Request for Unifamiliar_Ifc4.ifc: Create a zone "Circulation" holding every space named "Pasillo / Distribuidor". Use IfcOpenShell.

First a look at what the model holds.

```python
import ifcopenshell

model = ifcopenshell.open("Unifamiliar_Ifc4.ifc")
print(model.schema)
seen = {}
for space in model.by_type("IfcSpace"):
    seen[space.LongName] = seen.get(space.LongName, 0) + 1
for name, count in sorted(seen.items(), key=str):
    print(count, "x", name)
print("zones:", [z.Name for z in model.by_type("IfcZone")][:20])
```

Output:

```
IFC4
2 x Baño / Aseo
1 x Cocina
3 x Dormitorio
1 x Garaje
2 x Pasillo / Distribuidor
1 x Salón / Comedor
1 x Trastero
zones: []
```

```python
import ifcopenshell
import ifcopenshell.api.group
import ifcopenshell.api.root

model = ifcopenshell.open("Unifamiliar_Ifc4.ifc")

names = {"Pasillo / Distribuidor"}
spaces = [s for s in model.by_type("IfcSpace") if s.LongName in names]

zone = ifcopenshell.api.root.create_entity(model, ifc_class="IfcZone", name="Circulation")
ifcopenshell.api.group.assign_group(model, products=spaces, group=zone)
print(len(spaces), "spaces in", zone.Name)

model.write("Unifamiliar_Ifc4_v2.ifc")
```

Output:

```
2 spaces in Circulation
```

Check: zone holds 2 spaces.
